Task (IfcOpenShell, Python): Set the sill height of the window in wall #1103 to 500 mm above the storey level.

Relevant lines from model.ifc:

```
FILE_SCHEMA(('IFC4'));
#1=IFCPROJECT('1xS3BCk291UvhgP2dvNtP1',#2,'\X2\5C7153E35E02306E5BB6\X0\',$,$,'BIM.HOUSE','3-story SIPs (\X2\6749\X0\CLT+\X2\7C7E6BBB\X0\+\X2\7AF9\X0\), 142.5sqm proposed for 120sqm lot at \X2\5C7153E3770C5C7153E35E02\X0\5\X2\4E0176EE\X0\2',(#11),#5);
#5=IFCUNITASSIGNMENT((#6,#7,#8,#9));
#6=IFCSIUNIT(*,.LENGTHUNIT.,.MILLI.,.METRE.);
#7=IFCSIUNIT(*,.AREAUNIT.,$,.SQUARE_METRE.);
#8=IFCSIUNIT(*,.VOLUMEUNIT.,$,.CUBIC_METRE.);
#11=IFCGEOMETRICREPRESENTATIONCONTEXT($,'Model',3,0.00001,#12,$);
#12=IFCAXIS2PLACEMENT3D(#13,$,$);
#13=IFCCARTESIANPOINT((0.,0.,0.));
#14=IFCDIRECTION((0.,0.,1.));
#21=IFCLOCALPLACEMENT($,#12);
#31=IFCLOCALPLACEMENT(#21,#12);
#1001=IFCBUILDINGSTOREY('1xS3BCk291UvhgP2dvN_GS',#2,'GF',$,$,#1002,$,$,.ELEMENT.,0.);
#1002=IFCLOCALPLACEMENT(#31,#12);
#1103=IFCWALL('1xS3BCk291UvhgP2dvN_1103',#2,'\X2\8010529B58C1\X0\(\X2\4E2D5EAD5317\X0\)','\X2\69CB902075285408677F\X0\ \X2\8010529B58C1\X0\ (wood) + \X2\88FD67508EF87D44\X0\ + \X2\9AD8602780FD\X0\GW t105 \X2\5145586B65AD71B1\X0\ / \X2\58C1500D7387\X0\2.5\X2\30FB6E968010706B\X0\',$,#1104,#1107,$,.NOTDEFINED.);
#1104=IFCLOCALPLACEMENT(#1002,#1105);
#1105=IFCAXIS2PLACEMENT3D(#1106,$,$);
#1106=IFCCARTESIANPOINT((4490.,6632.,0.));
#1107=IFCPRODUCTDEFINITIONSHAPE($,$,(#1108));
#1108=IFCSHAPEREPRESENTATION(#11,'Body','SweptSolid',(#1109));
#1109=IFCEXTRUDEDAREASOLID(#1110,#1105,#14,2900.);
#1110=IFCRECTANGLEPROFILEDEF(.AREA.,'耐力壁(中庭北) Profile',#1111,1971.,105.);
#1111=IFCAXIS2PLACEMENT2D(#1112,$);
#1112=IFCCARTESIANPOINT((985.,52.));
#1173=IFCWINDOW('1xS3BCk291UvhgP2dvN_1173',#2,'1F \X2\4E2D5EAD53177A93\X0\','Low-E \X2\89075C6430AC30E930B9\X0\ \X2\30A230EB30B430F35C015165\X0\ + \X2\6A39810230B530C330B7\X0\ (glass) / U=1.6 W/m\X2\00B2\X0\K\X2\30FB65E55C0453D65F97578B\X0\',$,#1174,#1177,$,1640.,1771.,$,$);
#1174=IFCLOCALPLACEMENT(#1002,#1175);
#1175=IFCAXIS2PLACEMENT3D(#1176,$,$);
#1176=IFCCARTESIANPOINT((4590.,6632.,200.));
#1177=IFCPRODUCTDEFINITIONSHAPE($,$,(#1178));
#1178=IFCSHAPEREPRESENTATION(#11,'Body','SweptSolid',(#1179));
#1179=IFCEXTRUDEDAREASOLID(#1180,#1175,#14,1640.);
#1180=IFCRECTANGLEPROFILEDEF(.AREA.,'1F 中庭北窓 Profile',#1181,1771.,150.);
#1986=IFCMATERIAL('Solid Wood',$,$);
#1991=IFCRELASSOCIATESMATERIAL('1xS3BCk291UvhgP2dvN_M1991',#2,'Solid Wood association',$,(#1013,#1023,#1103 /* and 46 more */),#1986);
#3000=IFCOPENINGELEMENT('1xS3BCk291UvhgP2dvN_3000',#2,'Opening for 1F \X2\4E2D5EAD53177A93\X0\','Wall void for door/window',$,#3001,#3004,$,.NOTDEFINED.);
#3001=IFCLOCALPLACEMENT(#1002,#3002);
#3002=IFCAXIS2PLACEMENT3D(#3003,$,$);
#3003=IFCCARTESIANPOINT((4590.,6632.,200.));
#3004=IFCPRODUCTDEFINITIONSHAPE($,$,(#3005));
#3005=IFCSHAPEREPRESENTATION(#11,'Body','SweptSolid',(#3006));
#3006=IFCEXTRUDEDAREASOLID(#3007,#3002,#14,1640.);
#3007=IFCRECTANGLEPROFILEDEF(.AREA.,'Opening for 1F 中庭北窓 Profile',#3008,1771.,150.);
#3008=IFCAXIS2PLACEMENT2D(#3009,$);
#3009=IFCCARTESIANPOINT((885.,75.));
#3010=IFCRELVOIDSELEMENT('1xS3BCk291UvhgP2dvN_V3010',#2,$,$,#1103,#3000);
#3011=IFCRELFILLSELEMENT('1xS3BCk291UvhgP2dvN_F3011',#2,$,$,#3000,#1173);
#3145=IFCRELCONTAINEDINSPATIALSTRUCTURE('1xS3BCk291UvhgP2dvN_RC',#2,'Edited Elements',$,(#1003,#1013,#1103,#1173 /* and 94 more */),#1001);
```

```python
import numpy as np
import ifcopenshell
import ifcopenshell.api.geometry
import ifcopenshell.geom
import ifcopenshell.util.element
import ifcopenshell.util.placement
import ifcopenshell.util.shape
import ifcopenshell.util.unit

model = ifcopenshell.open("model.ifc")
unit_scale = ifcopenshell.util.unit.calculate_unit_scale(model)

window = model.by_id(1173)
opening = window.FillsVoids[0].RelatingOpeningElement
storey = ifcopenshell.util.element.get_container(window, ifc_class="IfcBuildingStorey")
level = ifcopenshell.util.placement.get_local_placement(storey.ObjectPlacement)[2, 3]

# The opening's origin need not be at the sill, so measure its lowest point.
shape = ifcopenshell.geom.create_shape(ifcopenshell.geom.settings(), opening)
bottom = ifcopenshell.util.shape.get_shape_bottom_elevation(shape, shape.geometry) / unit_scale
dz = level + 500.0 - bottom

shift = np.array([0.0, 0.0, dz])
# The window is not placed relative to its opening, so move both.
for product in (opening, window):
    matrix = ifcopenshell.util.placement.get_local_placement(product.ObjectPlacement)
    matrix[:3, 3] += shift
    ifcopenshell.api.geometry.edit_object_placement(model, product=product, matrix=matrix, is_si=False)

print(f"moved by {dz * unit_scale:+.3f} m")

model.write("model_v2.ifc")
```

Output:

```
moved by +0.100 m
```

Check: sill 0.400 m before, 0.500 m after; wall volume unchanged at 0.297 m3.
